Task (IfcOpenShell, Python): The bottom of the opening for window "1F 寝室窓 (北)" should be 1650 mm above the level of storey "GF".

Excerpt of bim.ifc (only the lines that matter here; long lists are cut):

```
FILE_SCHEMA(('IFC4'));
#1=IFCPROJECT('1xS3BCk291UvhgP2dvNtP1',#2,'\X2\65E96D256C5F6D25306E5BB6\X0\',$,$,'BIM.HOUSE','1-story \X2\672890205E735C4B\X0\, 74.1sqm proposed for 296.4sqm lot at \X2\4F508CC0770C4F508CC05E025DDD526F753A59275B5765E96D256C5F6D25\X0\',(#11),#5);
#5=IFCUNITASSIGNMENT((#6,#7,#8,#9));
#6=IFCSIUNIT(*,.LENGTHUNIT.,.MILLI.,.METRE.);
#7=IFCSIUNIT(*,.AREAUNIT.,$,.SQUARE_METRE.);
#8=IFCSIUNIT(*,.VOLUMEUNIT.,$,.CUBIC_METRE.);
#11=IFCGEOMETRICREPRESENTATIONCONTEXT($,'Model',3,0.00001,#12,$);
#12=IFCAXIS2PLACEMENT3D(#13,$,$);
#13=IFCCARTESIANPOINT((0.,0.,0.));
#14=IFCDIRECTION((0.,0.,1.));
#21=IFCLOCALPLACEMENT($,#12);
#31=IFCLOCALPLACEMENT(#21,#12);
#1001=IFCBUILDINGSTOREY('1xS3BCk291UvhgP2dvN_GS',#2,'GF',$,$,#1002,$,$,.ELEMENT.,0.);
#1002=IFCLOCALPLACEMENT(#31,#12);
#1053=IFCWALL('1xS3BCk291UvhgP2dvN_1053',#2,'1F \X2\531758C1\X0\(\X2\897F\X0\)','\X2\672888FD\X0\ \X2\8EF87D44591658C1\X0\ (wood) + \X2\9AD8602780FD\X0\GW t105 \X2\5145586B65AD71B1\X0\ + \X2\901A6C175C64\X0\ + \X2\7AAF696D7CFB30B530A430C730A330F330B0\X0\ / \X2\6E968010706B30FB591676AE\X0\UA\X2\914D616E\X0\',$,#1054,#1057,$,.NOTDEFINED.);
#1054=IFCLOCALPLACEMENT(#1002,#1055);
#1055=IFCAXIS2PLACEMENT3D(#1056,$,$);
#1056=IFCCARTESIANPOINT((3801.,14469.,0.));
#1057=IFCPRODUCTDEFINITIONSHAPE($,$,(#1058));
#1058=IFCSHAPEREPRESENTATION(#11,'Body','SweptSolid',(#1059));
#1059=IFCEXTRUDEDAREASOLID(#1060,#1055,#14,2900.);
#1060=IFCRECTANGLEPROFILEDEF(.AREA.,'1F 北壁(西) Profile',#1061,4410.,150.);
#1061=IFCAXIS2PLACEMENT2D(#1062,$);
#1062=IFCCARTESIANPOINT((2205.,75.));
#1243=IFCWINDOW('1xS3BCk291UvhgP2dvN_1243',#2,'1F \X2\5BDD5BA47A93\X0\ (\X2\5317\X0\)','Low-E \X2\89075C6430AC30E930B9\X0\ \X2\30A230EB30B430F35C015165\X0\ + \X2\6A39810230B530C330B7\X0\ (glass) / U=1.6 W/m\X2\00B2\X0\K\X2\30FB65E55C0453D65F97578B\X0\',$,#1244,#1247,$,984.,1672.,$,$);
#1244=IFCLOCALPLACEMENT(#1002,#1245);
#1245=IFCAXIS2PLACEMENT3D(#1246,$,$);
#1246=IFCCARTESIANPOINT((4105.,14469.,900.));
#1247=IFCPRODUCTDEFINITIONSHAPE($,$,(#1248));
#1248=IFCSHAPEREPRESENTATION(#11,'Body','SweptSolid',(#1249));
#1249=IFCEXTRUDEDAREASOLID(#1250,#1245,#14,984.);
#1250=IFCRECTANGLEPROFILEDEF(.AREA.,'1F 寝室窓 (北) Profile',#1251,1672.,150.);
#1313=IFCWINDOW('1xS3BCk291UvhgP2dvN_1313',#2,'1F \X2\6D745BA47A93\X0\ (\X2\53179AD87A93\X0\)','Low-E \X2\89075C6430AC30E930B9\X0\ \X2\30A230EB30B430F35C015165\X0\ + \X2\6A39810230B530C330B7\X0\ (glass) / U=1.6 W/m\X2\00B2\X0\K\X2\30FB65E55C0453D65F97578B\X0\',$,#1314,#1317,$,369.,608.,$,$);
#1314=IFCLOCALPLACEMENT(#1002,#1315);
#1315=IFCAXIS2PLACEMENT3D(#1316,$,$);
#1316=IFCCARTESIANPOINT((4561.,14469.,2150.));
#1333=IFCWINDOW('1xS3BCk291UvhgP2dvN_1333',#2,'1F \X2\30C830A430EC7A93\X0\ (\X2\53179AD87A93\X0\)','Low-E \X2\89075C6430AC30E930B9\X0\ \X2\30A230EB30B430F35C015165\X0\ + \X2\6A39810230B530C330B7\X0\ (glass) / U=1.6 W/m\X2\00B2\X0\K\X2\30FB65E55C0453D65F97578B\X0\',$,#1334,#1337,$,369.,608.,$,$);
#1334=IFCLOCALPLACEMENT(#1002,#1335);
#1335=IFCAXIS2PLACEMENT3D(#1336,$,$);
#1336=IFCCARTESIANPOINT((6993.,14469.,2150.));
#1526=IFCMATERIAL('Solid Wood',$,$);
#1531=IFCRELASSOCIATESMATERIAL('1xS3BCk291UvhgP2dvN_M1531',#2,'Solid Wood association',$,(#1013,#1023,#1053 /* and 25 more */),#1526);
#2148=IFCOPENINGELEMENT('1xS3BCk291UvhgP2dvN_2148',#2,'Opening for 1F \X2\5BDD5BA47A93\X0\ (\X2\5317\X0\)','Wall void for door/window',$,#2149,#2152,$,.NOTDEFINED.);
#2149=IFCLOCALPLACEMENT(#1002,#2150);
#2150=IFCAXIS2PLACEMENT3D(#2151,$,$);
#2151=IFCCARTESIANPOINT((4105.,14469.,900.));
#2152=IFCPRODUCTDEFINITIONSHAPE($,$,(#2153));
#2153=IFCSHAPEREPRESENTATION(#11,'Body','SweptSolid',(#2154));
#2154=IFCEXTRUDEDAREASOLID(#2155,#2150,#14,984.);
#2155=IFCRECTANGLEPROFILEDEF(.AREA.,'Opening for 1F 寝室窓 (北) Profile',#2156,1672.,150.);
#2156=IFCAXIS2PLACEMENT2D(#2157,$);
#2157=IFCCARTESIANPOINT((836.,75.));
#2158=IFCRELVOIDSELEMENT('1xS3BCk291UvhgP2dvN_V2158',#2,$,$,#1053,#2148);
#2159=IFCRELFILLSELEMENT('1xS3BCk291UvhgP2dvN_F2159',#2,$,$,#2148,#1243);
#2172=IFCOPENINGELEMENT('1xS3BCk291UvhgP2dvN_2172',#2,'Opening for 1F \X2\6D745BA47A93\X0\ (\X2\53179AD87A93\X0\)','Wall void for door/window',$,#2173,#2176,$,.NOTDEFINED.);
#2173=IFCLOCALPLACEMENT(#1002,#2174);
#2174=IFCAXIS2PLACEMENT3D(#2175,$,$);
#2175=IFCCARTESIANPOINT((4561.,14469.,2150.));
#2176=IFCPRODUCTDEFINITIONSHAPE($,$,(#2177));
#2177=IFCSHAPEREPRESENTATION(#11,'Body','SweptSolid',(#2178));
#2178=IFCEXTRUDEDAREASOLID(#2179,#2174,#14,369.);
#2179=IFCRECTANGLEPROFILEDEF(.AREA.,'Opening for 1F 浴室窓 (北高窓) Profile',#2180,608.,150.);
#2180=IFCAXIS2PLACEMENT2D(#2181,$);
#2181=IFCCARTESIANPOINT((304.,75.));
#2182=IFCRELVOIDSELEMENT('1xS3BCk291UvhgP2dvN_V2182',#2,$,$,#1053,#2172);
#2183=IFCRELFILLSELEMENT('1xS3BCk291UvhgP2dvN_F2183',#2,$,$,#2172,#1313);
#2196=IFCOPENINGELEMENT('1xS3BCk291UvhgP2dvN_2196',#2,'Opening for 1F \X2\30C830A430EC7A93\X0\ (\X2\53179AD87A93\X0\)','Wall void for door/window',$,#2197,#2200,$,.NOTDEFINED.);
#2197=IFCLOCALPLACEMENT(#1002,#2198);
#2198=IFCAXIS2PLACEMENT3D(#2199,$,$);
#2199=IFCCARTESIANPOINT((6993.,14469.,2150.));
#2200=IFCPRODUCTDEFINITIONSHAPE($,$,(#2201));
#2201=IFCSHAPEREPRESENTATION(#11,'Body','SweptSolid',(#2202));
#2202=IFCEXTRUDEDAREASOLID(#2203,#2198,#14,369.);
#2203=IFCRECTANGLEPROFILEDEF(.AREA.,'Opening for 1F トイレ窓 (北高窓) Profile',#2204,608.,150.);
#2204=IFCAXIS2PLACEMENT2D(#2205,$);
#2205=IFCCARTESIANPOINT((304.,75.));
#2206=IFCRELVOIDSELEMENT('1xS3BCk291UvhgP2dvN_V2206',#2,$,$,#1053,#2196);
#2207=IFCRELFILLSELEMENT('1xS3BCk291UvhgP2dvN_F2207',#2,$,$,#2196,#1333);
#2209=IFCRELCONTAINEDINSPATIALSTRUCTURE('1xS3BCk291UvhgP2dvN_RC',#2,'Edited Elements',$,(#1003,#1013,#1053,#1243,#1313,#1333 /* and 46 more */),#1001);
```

```python
import numpy as np
import ifcopenshell
import ifcopenshell.api.geometry
import ifcopenshell.geom
import ifcopenshell.util.element
import ifcopenshell.util.placement
import ifcopenshell.util.shape
import ifcopenshell.util.unit

model = ifcopenshell.open("bim.ifc")
unit_scale = ifcopenshell.util.unit.calculate_unit_scale(model)

window = model.by_guid("1xS3BCk291UvhgP2dvN_1243")
opening = window.FillsVoids[0].RelatingOpeningElement
storey = ifcopenshell.util.element.get_container(window, ifc_class="IfcBuildingStorey")
level = ifcopenshell.util.placement.get_local_placement(storey.ObjectPlacement)[2, 3]

# The opening's origin need not be at the sill, so measure its lowest point.
shape = ifcopenshell.geom.create_shape(ifcopenshell.geom.settings(), opening)
bottom = ifcopenshell.util.shape.get_shape_bottom_elevation(shape, shape.geometry) / unit_scale
dz = level + 1.65 / unit_scale - bottom

shift = np.array([0.0, 0.0, dz])
# The window is not placed relative to its opening, so move both.
for product in (opening, window):
    matrix = ifcopenshell.util.placement.get_local_placement(product.ObjectPlacement)
    matrix[:3, 3] += shift
    ifcopenshell.api.geometry.edit_object_placement(model, product=product, matrix=matrix, is_si=False)

print(f"moved by {dz * unit_scale:+.3f} m")

model.write("bim_updated.ifc")
```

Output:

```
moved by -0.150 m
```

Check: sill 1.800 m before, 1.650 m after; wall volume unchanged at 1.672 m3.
